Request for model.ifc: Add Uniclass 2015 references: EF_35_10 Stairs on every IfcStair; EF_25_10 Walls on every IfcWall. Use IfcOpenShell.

First a look at what the model holds.

```python
import ifcopenshell

model = ifcopenshell.open("model.ifc")
print(model.schema)
print("classifications:", [c.Name for c in model.by_type("IfcClassification")])
for ifc_class in ("IfcDoor", "IfcRoof", "IfcStair", "IfcWall", "IfcWindow"):
    print(ifc_class, len(model.by_type(ifc_class)))
```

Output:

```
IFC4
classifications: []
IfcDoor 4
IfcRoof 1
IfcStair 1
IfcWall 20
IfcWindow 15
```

```python
import ifcopenshell
import ifcopenshell.api.classification

model = ifcopenshell.open("model.ifc")

system = ifcopenshell.api.classification.add_classification(model, classification="Uniclass 2015")

codes = {
    "IfcStair": ("EF_35_10", "Stairs"),
    "IfcWall": ("EF_25_10", "Walls"),
}
for ifc_class, (code, name) in codes.items():
    products = model.by_type(ifc_class)
    ifcopenshell.api.classification.add_reference(
        model, products=products, classification=system, identification=code, name=name
    )
    print(code, len(products))

model.write("model_updated.ifc")
```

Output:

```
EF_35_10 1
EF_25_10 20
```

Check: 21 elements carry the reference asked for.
